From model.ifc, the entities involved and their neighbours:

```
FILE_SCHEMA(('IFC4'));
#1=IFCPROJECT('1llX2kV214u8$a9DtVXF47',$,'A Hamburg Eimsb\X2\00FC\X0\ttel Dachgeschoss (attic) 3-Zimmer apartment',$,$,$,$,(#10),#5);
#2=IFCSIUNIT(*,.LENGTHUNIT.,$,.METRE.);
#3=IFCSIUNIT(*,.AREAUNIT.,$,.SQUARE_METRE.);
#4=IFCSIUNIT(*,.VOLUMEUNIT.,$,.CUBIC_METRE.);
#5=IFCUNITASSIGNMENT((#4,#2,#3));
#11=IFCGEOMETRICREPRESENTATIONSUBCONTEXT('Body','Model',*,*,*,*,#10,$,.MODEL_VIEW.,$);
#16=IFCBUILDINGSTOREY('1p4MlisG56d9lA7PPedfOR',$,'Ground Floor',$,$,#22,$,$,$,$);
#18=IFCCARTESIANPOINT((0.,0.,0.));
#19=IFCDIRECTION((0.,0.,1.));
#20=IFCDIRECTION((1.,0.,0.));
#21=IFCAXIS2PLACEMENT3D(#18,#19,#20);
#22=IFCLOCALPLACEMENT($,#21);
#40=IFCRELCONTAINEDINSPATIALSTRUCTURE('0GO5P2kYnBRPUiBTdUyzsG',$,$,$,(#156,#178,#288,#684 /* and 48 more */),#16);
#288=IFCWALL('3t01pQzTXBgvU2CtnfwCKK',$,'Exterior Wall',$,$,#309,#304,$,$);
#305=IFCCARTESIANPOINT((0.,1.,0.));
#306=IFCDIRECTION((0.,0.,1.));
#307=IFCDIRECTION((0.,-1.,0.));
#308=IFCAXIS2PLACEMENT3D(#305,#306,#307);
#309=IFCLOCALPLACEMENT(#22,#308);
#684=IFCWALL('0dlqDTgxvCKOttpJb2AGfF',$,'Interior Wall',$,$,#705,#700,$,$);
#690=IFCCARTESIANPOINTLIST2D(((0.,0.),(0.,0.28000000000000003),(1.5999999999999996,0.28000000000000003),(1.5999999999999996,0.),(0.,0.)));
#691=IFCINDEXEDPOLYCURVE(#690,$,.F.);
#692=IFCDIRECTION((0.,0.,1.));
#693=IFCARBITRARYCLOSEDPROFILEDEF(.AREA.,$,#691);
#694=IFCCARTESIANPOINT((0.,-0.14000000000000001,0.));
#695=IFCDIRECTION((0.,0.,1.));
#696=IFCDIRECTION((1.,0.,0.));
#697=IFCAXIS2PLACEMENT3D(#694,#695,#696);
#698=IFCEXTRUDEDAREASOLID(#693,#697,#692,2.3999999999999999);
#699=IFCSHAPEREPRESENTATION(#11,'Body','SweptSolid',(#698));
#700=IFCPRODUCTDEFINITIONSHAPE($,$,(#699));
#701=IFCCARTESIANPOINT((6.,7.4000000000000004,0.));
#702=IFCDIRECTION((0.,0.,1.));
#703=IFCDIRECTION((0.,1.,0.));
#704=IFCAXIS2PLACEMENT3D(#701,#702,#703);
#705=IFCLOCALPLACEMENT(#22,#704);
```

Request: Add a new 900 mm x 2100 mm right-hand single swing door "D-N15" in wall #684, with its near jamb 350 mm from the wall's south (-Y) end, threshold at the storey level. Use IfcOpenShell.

```python
import numpy as np
import ifcopenshell
import ifcopenshell.api.feature
import ifcopenshell.api.geometry
import ifcopenshell.api.root
import ifcopenshell.api.spatial
import ifcopenshell.geom
import ifcopenshell.util.element
import ifcopenshell.util.placement
import ifcopenshell.util.representation
import ifcopenshell.util.shape
import ifcopenshell.util.unit

model = ifcopenshell.open("model.ifc")
unit_scale = ifcopenshell.util.unit.calculate_unit_scale(model)
settings = ifcopenshell.geom.settings()


def volume(element):
    """Net volume in cubic metres, openings subtracted."""
    shape = ifcopenshell.geom.create_shape(settings, element)
    return ifcopenshell.util.shape.get_volume(shape.geometry)


wall = model.by_id(684)
storey = ifcopenshell.util.element.get_container(wall, ifc_class="IfcBuildingStorey")
context = ifcopenshell.util.representation.get_context(model, "Model", "Body", "MODEL_VIEW")
before = volume(wall)

width, height, from_end, sill = 0.9, 2.1, 0.35, 0.0  # metres

# The wall runs along its own X axis, and the end named is its -X end.
wall_shape = ifcopenshell.geom.create_shape(settings, wall)
x, y, z = ifcopenshell.util.shape.get_vertices(wall_shape.geometry).T
start = x.min() + from_end
face, thickness = float(y.min()), float(y.max() - y.min())
wall_matrix = ifcopenshell.util.placement.get_local_placement(wall.ObjectPlacement)
level = ifcopenshell.util.placement.get_local_placement(storey.ObjectPlacement)[2, 3]


def in_wall(x, y):
    """Placement at x, y metres in the wall's axes, at sill height."""
    matrix = wall_matrix.copy()
    matrix[:, 3] = wall_matrix @ np.array([x / unit_scale, y / unit_scale, 0.0, 1.0])
    matrix[2, 3] = level + sill / unit_scale
    return matrix


# Opening: a box that overshoots both wall faces by 50 mm.
opening = ifcopenshell.api.root.create_entity(model, ifc_class="IfcOpeningElement", predefined_type="OPENING")
box = ifcopenshell.api.geometry.add_wall_representation(
    model, context=context, length=width, height=height, thickness=thickness + 0.1
)
ifcopenshell.api.geometry.assign_representation(model, product=opening, representation=box)
ifcopenshell.api.geometry.edit_object_placement(model, product=opening, matrix=in_wall(start, face - 0.05), is_si=False)
ifcopenshell.api.feature.add_feature(model, feature=opening, element=wall)

door = ifcopenshell.api.root.create_entity(model, ifc_class="IfcDoor", name="D-N15", predefined_type="DOOR")
door.OverallWidth, door.OverallHeight = width / unit_scale, height / unit_scale
door.OperationType = "SINGLE_SWING_RIGHT"
body = ifcopenshell.api.geometry.add_door_representation(
    model,
    context=context,
    overall_width=door.OverallWidth,
    overall_height=door.OverallHeight,
    operation_type="SINGLE_SWING_RIGHT",
    lining_properties={"LiningDepth": thickness / unit_scale, "ThresholdDepth": thickness / unit_scale},
)
ifcopenshell.api.geometry.assign_representation(model, product=door, representation=body)
ifcopenshell.api.spatial.assign_container(model, products=[door], relating_structure=storey)
ifcopenshell.api.feature.add_filling(model, opening=opening, element=door)

# The lining spans the wall, so the door starts at the wall face.
ifcopenshell.api.geometry.edit_object_placement(model, product=door, matrix=in_wall(start, face), is_si=False)

after = volume(wall)

print(f"wall volume {before:.3f} -> {after:.3f} m3")

model.write("model_rev.ifc")
```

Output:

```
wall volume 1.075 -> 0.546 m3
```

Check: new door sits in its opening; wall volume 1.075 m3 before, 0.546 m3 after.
